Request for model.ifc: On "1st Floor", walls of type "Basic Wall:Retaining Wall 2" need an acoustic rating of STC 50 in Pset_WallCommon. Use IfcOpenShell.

First a look at what the model holds.

```python
import ifcopenshell
import ifcopenshell.util.element

model = ifcopenshell.open("model.ifc")
print(model.schema)
storey = next(s for s in model.by_type("IfcBuildingStorey") if s.Name == "1st Floor")
walls = [e for e in ifcopenshell.util.element.get_decomposition(storey) if e.is_a("IfcWall")]
seen = {}
for e in walls:
    element_type = ifcopenshell.util.element.get_type(e)
    key = (element_type.Name if element_type != e and element_type else None, ifcopenshell.util.element.get_pset(e, "Pset_WallCommon", "AcousticRating"))
    seen[key] = seen.get(key, 0) + 1
for (name, value), count in sorted(seen.items(), key=str):
    print(count, "x", name, "|", value)
```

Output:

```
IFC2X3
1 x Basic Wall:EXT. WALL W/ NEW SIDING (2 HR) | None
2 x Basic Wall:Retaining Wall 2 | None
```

```python
import ifcopenshell
import ifcopenshell.api.pset
import ifcopenshell.util.element

model = ifcopenshell.open("model.ifc")

storey = next(s for s in model.by_type("IfcBuildingStorey") if s.Name == "1st Floor")
walls = [e for e in ifcopenshell.util.element.get_decomposition(storey) if e.is_a("IfcWall")]

count = 0
for e in walls:
    element_type = ifcopenshell.util.element.get_type(e)
    if element_type in (None, e) or element_type.Name != "Basic Wall:Retaining Wall 2":
        continue
    # add_pset returns the element's existing set when there is one.
    pset = ifcopenshell.api.pset.add_pset(model, product=e, name="Pset_WallCommon")
    ifcopenshell.api.pset.edit_pset(model, pset=pset, properties={"AcousticRating": "STC 50"})
    count += 1

print(count, "walls updated")

model.write("model_edited.ifc")
```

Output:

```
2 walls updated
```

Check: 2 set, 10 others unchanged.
